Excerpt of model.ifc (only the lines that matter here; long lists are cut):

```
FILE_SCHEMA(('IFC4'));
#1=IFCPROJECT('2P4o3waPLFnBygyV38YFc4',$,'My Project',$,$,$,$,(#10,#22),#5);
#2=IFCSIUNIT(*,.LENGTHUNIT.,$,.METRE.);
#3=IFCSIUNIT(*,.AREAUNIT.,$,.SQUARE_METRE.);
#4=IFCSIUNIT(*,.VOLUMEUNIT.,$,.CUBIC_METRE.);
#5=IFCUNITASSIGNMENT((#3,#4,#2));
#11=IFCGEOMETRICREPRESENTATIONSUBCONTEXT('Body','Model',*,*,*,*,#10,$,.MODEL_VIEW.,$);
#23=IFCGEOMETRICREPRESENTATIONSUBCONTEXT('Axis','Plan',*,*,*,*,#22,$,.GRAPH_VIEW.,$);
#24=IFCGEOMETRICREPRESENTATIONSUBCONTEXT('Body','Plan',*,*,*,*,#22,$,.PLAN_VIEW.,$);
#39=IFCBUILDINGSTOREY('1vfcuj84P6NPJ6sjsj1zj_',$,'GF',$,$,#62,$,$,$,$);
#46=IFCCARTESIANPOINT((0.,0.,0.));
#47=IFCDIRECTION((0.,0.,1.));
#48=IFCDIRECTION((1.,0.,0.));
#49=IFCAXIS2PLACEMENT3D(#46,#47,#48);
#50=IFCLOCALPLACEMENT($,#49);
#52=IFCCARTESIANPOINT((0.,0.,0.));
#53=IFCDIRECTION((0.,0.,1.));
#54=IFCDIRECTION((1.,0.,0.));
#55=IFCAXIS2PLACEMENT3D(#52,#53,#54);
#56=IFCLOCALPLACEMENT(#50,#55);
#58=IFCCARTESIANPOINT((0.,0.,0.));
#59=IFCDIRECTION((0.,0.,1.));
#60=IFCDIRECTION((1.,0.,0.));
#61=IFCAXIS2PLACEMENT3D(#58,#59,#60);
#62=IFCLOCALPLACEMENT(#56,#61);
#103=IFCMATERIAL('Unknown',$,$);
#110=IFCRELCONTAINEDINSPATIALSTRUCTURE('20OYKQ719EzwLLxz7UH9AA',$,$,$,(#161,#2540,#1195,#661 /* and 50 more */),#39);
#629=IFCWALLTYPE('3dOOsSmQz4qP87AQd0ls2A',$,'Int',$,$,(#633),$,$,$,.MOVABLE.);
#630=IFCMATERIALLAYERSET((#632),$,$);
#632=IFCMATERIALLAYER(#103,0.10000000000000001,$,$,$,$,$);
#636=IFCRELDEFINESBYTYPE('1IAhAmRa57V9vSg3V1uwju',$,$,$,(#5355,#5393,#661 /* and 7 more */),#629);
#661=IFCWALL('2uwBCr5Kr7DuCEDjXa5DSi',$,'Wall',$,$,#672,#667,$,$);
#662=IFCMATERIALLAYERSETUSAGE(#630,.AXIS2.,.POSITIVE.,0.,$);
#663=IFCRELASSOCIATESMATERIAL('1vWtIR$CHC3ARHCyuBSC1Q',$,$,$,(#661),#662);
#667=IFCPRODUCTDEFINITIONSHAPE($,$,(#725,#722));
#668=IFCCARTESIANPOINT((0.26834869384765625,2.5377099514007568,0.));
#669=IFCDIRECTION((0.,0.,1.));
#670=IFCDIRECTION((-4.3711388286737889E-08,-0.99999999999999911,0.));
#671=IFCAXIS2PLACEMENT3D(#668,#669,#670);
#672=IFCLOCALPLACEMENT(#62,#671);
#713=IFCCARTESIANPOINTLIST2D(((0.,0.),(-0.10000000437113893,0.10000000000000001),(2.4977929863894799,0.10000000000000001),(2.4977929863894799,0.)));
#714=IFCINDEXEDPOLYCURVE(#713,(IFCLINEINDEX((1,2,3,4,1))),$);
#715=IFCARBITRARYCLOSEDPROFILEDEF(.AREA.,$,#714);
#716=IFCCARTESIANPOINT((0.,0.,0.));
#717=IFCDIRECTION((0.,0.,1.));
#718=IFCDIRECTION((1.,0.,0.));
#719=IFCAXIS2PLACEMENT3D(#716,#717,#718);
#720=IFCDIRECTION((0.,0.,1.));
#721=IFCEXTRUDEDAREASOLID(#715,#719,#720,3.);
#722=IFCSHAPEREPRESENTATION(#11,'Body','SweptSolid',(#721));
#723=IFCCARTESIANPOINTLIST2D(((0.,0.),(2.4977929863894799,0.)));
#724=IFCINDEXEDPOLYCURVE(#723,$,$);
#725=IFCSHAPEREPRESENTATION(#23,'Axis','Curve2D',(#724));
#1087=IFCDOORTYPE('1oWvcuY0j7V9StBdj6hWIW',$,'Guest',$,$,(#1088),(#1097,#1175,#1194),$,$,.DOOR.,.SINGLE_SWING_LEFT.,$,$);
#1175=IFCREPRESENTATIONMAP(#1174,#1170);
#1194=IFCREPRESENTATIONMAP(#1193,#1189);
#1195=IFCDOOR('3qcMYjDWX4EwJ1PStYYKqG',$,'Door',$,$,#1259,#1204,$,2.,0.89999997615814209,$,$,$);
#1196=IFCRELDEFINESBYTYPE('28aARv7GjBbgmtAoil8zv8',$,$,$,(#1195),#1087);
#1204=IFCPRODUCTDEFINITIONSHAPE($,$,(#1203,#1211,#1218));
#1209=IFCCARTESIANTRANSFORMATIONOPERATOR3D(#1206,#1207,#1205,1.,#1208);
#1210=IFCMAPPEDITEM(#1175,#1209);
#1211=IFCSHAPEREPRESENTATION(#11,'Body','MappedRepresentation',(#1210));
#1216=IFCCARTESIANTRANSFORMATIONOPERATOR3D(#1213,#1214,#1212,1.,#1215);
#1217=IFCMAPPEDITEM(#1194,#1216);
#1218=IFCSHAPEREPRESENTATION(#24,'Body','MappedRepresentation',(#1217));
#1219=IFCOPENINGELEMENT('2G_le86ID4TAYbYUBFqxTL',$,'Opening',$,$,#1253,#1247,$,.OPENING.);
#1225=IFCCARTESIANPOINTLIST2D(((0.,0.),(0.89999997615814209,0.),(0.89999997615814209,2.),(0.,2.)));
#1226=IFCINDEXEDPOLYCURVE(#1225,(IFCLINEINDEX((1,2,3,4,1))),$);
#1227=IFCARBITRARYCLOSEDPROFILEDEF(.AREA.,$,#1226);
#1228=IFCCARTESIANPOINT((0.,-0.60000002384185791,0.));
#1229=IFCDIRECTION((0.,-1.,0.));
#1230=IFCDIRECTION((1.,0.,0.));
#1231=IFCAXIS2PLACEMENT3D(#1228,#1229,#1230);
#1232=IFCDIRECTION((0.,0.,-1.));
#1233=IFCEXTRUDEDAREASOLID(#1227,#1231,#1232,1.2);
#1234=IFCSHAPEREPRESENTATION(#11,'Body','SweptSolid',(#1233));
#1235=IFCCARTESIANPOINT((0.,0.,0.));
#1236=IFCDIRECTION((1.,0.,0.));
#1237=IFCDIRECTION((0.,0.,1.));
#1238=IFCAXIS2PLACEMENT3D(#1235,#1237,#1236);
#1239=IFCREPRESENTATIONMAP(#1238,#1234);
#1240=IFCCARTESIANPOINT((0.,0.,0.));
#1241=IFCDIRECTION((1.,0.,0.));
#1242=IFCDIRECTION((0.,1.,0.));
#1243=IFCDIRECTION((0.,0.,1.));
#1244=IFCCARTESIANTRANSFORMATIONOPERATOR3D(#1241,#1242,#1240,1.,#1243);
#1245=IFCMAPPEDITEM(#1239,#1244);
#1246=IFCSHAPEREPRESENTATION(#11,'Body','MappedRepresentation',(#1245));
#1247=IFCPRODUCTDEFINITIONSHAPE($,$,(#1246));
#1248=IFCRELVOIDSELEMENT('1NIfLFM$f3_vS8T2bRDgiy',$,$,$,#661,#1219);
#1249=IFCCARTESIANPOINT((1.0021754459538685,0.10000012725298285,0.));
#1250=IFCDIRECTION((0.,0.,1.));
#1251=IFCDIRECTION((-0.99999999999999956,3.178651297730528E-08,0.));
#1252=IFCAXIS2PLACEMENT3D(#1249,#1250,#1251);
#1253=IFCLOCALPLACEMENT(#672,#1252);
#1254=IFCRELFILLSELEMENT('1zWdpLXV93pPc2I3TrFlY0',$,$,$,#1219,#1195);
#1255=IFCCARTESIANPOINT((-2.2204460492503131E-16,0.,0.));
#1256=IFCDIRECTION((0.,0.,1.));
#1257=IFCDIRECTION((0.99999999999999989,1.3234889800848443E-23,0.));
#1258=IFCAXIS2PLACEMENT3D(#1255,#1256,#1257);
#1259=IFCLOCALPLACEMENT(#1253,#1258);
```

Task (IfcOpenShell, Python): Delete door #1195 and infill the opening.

```python
import ifcopenshell
import ifcopenshell.api.feature
import ifcopenshell.api.root
import ifcopenshell.geom
import ifcopenshell.util.shape

model = ifcopenshell.open("model.ifc")
settings = ifcopenshell.geom.settings()


def volume(element):
    """Net volume in cubic metres, openings subtracted."""
    shape = ifcopenshell.geom.create_shape(settings, element)
    return ifcopenshell.util.shape.get_volume(shape.geometry)


door = model.by_guid("3qcMYjDWX4EwJ1PStYYKqG")
opening = door.FillsVoids[0].RelatingOpeningElement
wall = opening.VoidsElements[0].RelatingBuildingElement
before = volume(wall)

ifcopenshell.api.root.remove_product(model, product=door)
ifcopenshell.api.feature.remove_feature(model, feature=opening)

after = volume(wall)

print(f"wall volume {before:.3f} -> {after:.3f} m3")

model.write("model_edited.ifc")
```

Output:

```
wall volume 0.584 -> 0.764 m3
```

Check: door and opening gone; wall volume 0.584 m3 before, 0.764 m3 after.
